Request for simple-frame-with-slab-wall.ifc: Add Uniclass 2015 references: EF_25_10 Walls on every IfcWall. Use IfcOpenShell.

First a look at what the model holds.

```python
import ifcopenshell

model = ifcopenshell.open("simple-frame-with-slab-wall.ifc")
print(model.schema)
print("classifications:", [c.Name for c in model.by_type("IfcClassification")])
for ifc_class in ("IfcDoor", "IfcRoof", "IfcStair", "IfcWall", "IfcWindow"):
    print(ifc_class, len(model.by_type(ifc_class)))
```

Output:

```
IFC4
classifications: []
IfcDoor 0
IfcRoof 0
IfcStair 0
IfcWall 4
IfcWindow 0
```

```python
import ifcopenshell
import ifcopenshell.api.classification

model = ifcopenshell.open("simple-frame-with-slab-wall.ifc")

system = ifcopenshell.api.classification.add_classification(model, classification="Uniclass 2015")

codes = {
    "IfcWall": ("EF_25_10", "Walls"),
}
for ifc_class, (code, name) in codes.items():
    products = model.by_type(ifc_class)
    ifcopenshell.api.classification.add_reference(
        model, products=products, classification=system, identification=code, name=name
    )
    print(code, len(products))

model.write("simple-frame-with-slab-wall_updated.ifc")
```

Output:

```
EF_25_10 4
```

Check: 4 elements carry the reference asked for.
